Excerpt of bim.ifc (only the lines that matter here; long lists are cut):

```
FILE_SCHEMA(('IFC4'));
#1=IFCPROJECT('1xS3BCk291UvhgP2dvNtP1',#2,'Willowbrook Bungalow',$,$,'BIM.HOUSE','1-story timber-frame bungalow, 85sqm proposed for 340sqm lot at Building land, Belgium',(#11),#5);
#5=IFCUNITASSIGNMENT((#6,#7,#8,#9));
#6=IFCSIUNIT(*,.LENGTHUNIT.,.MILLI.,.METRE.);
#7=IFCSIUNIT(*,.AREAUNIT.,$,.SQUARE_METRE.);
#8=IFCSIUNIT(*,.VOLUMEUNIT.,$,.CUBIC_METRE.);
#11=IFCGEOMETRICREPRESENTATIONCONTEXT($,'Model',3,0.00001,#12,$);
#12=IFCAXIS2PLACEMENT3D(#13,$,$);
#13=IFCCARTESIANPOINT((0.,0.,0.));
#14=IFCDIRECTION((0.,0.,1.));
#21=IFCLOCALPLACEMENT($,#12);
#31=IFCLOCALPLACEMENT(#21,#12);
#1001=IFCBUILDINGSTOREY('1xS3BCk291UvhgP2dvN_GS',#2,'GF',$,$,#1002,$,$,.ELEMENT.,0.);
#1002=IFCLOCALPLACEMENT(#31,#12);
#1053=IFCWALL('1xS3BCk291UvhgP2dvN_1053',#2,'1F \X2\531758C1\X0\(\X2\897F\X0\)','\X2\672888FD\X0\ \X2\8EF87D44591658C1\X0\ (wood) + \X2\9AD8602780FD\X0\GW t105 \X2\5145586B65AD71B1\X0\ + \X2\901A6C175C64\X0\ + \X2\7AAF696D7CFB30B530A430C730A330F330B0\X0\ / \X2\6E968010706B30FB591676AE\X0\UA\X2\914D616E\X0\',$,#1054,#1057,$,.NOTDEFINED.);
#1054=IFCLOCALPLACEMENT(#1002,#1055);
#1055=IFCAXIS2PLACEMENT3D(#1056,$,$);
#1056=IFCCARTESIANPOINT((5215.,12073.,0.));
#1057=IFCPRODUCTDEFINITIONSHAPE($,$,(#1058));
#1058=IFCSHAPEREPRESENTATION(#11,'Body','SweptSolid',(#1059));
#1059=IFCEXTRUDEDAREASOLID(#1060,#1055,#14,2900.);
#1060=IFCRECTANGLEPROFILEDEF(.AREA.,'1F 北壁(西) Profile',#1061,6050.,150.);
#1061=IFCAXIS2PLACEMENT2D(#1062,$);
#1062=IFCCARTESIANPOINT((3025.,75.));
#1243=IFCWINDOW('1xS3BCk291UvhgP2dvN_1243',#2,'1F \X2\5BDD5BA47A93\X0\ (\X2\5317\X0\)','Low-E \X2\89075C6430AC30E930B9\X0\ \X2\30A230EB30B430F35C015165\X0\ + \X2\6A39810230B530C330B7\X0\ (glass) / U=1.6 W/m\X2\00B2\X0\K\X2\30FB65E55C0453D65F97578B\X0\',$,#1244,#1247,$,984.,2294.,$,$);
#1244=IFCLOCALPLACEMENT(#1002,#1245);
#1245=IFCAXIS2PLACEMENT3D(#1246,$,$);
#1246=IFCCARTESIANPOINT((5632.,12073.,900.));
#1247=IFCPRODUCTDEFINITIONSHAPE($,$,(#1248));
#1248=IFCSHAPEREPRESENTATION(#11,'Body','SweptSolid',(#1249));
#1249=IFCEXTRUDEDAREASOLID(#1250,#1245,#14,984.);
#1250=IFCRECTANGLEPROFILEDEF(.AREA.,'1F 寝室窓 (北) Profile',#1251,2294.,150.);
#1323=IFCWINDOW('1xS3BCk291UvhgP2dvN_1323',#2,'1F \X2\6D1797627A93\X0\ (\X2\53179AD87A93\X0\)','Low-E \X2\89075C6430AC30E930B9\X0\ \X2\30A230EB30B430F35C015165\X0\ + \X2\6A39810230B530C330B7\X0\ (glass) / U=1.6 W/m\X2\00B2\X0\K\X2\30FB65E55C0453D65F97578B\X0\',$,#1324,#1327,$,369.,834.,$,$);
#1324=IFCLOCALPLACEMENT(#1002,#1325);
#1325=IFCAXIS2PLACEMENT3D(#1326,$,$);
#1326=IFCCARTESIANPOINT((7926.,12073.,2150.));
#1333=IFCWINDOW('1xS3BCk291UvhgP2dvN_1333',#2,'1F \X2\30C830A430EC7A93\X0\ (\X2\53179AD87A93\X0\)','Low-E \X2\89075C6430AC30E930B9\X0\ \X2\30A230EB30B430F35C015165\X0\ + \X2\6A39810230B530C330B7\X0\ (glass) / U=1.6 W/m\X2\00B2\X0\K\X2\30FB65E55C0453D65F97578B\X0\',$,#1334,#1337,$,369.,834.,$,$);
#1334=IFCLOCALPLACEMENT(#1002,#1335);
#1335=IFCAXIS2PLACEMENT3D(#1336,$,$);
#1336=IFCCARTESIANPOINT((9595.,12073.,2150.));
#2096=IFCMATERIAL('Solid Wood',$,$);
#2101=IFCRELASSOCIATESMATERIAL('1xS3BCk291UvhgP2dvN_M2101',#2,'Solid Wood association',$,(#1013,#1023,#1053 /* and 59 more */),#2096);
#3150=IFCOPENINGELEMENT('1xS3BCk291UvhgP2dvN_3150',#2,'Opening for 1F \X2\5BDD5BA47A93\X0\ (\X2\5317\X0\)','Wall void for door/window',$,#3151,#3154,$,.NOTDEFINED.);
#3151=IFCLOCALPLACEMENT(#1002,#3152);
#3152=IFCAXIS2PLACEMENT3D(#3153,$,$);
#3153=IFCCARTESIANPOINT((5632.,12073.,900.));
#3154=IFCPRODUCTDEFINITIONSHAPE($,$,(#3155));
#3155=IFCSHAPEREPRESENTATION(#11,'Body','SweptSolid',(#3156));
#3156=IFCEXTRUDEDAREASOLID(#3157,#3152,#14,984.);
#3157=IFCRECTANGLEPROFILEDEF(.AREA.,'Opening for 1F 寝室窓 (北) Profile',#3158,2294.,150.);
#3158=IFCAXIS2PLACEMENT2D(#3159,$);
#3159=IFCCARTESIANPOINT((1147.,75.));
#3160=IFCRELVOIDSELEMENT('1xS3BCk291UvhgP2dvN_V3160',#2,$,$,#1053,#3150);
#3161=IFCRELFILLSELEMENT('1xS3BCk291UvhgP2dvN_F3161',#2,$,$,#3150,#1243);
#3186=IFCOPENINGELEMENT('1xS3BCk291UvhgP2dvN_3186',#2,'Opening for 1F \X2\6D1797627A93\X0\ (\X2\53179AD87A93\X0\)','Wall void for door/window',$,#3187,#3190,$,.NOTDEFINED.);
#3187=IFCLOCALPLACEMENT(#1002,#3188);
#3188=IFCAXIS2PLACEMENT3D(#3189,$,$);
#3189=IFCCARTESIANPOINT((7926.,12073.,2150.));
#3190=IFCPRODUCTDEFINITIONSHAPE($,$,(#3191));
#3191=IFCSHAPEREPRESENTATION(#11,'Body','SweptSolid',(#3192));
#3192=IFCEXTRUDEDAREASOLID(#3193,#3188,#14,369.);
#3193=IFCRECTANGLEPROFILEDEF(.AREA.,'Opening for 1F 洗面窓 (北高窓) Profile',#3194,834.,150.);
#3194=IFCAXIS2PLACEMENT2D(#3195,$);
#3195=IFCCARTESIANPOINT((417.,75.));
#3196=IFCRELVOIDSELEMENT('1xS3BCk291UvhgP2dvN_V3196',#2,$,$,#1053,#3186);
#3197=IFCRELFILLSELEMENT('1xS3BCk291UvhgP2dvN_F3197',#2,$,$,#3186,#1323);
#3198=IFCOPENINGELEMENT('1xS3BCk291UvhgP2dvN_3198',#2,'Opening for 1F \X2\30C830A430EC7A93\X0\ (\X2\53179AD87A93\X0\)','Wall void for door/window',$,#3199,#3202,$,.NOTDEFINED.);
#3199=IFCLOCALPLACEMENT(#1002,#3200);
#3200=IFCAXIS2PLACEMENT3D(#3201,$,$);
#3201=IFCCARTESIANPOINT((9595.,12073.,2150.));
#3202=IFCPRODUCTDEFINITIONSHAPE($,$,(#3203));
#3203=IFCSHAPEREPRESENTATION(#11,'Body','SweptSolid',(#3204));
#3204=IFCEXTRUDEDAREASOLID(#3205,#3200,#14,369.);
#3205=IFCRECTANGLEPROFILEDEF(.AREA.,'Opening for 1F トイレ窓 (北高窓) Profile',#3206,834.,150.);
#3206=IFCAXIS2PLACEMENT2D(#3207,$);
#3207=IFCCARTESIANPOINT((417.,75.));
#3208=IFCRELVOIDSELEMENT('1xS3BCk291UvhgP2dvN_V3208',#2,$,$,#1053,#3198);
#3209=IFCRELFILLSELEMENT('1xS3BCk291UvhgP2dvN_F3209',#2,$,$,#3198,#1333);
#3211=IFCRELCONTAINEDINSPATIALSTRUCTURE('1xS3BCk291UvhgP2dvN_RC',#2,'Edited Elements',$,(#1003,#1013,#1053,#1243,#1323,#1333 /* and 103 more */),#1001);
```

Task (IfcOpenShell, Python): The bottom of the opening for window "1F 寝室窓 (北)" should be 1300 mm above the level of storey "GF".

```python
import numpy as np
import ifcopenshell
import ifcopenshell.api.geometry
import ifcopenshell.geom
import ifcopenshell.util.element
import ifcopenshell.util.placement
import ifcopenshell.util.shape
import ifcopenshell.util.unit

model = ifcopenshell.open("bim.ifc")
unit_scale = ifcopenshell.util.unit.calculate_unit_scale(model)

window = model.by_guid("1xS3BCk291UvhgP2dvN_1243")
opening = window.FillsVoids[0].RelatingOpeningElement
storey = ifcopenshell.util.element.get_container(window, ifc_class="IfcBuildingStorey")
level = ifcopenshell.util.placement.get_local_placement(storey.ObjectPlacement)[2, 3]

# The opening's origin need not be at the sill, so measure its lowest point.
shape = ifcopenshell.geom.create_shape(ifcopenshell.geom.settings(), opening)
bottom = ifcopenshell.util.shape.get_shape_bottom_elevation(shape, shape.geometry) / unit_scale
dz = level + 1300.0 - bottom

shift = np.array([0.0, 0.0, dz])
# The window is not placed relative to its opening, so move both.
for product in (opening, window):
    matrix = ifcopenshell.util.placement.get_local_placement(product.ObjectPlacement)
    matrix[:3, 3] += shift
    ifcopenshell.api.geometry.edit_object_placement(model, product=product, matrix=matrix, is_si=False)

print(f"moved by {dz * unit_scale:+.3f} m")

model.write("bim_updated.ifc")
```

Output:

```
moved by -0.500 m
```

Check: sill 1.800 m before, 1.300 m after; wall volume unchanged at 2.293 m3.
